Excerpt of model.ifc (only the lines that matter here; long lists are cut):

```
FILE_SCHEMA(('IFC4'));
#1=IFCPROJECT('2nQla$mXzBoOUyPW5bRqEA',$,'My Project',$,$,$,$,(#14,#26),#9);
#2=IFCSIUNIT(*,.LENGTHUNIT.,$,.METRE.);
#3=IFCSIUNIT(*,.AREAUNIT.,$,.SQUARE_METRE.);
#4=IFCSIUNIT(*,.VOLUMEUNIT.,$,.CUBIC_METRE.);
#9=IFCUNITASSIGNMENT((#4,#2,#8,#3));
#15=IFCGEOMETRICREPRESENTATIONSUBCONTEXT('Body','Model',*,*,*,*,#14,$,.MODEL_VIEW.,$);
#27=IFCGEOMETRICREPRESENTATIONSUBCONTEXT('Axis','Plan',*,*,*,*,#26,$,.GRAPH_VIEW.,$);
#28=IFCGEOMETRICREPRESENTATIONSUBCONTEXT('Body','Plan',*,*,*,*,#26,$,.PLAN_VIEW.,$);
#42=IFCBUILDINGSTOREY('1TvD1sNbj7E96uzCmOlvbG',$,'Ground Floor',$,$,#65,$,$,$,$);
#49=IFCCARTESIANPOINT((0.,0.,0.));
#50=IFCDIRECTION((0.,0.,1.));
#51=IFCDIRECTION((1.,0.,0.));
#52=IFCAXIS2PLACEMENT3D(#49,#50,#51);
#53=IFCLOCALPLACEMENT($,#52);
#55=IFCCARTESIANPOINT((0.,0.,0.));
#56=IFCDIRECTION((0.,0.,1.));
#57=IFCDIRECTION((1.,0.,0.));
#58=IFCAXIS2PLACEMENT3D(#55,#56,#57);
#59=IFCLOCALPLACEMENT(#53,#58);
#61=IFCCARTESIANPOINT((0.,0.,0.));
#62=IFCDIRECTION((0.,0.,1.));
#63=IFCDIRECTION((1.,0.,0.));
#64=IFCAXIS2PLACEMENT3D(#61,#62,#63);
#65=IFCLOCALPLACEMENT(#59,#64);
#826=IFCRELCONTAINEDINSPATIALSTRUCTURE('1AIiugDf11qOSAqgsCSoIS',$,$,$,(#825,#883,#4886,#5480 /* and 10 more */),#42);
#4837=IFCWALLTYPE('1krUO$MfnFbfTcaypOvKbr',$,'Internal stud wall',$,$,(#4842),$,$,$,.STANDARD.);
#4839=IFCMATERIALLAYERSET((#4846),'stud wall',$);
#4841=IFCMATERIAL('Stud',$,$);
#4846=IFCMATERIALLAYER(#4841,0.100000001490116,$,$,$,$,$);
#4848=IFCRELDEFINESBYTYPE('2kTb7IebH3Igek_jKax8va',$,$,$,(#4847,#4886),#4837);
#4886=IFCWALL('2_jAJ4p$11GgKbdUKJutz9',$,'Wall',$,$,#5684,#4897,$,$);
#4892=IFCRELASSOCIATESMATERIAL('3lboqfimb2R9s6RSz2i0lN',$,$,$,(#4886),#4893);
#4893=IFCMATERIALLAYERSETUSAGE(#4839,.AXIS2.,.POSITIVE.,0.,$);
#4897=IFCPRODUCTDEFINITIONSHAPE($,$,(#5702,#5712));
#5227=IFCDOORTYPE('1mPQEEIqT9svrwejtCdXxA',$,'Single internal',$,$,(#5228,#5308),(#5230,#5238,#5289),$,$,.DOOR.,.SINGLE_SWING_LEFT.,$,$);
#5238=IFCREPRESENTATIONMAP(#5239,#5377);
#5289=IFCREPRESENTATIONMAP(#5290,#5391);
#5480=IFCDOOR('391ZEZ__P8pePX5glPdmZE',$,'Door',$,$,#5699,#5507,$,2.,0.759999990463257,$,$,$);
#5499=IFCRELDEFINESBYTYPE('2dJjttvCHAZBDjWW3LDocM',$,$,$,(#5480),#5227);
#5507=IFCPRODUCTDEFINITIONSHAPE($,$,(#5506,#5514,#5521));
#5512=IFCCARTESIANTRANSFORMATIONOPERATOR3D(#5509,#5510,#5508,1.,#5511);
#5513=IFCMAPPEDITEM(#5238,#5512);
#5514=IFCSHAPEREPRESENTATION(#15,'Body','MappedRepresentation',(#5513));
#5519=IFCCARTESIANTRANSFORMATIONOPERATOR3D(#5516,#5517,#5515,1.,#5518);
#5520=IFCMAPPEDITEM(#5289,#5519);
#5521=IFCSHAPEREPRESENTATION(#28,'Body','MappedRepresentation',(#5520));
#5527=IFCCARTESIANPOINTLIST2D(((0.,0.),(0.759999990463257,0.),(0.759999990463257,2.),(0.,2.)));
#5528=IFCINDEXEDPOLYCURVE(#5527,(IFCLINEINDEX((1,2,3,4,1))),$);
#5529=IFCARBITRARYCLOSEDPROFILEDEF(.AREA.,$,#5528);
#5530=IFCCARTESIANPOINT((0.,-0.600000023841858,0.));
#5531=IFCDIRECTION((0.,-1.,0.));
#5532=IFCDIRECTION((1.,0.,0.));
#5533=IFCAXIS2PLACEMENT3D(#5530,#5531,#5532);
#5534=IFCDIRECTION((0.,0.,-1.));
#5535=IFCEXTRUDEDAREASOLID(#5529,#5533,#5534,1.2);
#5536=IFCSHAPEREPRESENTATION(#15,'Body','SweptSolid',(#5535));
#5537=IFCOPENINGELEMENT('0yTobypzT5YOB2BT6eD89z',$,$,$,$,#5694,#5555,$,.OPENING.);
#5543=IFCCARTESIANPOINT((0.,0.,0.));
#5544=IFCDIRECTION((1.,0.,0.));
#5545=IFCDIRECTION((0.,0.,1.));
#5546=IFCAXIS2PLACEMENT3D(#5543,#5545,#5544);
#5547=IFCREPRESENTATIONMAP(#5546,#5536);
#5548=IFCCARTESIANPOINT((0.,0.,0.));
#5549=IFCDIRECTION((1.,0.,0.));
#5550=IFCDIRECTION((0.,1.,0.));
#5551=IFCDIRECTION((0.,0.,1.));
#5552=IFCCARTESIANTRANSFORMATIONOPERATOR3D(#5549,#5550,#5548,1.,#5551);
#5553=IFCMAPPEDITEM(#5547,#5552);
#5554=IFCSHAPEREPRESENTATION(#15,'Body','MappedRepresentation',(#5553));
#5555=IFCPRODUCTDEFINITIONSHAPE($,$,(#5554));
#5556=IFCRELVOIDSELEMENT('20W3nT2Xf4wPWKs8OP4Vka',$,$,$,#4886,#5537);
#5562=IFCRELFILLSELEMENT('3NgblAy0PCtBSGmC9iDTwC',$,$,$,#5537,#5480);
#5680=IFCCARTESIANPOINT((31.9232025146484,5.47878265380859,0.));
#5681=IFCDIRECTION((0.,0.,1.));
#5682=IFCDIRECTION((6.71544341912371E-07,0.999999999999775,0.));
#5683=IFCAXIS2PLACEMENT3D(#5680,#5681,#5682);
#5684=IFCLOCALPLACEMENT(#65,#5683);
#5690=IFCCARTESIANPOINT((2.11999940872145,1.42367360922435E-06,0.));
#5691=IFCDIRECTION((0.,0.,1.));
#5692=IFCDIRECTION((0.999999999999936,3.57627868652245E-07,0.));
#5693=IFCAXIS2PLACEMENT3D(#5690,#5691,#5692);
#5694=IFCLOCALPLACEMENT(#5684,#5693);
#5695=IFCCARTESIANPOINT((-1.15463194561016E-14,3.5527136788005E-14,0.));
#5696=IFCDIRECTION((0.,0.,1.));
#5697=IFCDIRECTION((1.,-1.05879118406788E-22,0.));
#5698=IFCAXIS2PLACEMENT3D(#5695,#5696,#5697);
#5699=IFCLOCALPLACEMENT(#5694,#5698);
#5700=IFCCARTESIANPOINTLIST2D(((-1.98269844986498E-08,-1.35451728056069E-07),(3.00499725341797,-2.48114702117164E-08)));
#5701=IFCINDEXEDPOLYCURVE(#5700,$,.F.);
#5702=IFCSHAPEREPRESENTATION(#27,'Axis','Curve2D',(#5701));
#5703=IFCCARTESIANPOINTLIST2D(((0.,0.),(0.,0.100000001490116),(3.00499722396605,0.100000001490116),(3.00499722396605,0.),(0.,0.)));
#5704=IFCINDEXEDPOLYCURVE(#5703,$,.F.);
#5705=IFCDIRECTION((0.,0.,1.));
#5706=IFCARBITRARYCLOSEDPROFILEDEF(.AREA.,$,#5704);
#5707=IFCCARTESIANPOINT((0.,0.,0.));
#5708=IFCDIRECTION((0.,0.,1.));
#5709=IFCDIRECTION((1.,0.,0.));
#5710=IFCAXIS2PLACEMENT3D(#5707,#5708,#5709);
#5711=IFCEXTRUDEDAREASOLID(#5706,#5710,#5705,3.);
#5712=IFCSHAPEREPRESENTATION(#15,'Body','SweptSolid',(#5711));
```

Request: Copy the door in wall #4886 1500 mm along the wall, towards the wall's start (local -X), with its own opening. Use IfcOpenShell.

```python
import ifcopenshell
import ifcopenshell.api.feature
import ifcopenshell.api.geometry
import ifcopenshell.api.root
import ifcopenshell.geom
import ifcopenshell.util.element
import ifcopenshell.util.placement
import ifcopenshell.util.shape
import ifcopenshell.util.unit

model = ifcopenshell.open("model.ifc")
unit_scale = ifcopenshell.util.unit.calculate_unit_scale(model)
settings = ifcopenshell.geom.settings()


def volume(element):
    """Net volume in cubic metres, openings subtracted."""
    shape = ifcopenshell.geom.create_shape(settings, element)
    return ifcopenshell.util.shape.get_volume(shape.geometry)


door = model.by_guid("391ZEZ__P8pePX5glPdmZE")
opening = door.FillsVoids[0].RelatingOpeningElement
wall = opening.VoidsElements[0].RelatingBuildingElement
before = volume(wall)
shift = ifcopenshell.util.placement.get_local_placement(wall.ObjectPlacement)[:3, 0] * -1.5 / unit_scale

# copy_class copies the void relationship, type, container and properties, but no geometry.
new_opening = ifcopenshell.api.root.copy_class(model, product=opening)
new_opening.Representation = ifcopenshell.util.element.copy_deep(
    model, opening.Representation, exclude=["IfcGeometricRepresentationContext", "IfcRepresentationMap"]
)
new_door = ifcopenshell.api.root.copy_class(model, product=door)
new_door.Representation = ifcopenshell.util.element.copy_deep(
    model, door.Representation, exclude=["IfcGeometricRepresentationContext", "IfcRepresentationMap"]
)
ifcopenshell.api.feature.add_filling(model, opening=new_opening, element=new_door)

for old, new in ((opening, new_opening), (door, new_door)):
    matrix = ifcopenshell.util.placement.get_local_placement(old.ObjectPlacement)
    matrix[:3, 3] += shift
    ifcopenshell.api.geometry.edit_object_placement(model, product=new, matrix=matrix, is_si=False)

after = volume(wall)

print(f"wall volume {before:.3f} -> {after:.3f} m3")

model.write("model-out.ifc")
```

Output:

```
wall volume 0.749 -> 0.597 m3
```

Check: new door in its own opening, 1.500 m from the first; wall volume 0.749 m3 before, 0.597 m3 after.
